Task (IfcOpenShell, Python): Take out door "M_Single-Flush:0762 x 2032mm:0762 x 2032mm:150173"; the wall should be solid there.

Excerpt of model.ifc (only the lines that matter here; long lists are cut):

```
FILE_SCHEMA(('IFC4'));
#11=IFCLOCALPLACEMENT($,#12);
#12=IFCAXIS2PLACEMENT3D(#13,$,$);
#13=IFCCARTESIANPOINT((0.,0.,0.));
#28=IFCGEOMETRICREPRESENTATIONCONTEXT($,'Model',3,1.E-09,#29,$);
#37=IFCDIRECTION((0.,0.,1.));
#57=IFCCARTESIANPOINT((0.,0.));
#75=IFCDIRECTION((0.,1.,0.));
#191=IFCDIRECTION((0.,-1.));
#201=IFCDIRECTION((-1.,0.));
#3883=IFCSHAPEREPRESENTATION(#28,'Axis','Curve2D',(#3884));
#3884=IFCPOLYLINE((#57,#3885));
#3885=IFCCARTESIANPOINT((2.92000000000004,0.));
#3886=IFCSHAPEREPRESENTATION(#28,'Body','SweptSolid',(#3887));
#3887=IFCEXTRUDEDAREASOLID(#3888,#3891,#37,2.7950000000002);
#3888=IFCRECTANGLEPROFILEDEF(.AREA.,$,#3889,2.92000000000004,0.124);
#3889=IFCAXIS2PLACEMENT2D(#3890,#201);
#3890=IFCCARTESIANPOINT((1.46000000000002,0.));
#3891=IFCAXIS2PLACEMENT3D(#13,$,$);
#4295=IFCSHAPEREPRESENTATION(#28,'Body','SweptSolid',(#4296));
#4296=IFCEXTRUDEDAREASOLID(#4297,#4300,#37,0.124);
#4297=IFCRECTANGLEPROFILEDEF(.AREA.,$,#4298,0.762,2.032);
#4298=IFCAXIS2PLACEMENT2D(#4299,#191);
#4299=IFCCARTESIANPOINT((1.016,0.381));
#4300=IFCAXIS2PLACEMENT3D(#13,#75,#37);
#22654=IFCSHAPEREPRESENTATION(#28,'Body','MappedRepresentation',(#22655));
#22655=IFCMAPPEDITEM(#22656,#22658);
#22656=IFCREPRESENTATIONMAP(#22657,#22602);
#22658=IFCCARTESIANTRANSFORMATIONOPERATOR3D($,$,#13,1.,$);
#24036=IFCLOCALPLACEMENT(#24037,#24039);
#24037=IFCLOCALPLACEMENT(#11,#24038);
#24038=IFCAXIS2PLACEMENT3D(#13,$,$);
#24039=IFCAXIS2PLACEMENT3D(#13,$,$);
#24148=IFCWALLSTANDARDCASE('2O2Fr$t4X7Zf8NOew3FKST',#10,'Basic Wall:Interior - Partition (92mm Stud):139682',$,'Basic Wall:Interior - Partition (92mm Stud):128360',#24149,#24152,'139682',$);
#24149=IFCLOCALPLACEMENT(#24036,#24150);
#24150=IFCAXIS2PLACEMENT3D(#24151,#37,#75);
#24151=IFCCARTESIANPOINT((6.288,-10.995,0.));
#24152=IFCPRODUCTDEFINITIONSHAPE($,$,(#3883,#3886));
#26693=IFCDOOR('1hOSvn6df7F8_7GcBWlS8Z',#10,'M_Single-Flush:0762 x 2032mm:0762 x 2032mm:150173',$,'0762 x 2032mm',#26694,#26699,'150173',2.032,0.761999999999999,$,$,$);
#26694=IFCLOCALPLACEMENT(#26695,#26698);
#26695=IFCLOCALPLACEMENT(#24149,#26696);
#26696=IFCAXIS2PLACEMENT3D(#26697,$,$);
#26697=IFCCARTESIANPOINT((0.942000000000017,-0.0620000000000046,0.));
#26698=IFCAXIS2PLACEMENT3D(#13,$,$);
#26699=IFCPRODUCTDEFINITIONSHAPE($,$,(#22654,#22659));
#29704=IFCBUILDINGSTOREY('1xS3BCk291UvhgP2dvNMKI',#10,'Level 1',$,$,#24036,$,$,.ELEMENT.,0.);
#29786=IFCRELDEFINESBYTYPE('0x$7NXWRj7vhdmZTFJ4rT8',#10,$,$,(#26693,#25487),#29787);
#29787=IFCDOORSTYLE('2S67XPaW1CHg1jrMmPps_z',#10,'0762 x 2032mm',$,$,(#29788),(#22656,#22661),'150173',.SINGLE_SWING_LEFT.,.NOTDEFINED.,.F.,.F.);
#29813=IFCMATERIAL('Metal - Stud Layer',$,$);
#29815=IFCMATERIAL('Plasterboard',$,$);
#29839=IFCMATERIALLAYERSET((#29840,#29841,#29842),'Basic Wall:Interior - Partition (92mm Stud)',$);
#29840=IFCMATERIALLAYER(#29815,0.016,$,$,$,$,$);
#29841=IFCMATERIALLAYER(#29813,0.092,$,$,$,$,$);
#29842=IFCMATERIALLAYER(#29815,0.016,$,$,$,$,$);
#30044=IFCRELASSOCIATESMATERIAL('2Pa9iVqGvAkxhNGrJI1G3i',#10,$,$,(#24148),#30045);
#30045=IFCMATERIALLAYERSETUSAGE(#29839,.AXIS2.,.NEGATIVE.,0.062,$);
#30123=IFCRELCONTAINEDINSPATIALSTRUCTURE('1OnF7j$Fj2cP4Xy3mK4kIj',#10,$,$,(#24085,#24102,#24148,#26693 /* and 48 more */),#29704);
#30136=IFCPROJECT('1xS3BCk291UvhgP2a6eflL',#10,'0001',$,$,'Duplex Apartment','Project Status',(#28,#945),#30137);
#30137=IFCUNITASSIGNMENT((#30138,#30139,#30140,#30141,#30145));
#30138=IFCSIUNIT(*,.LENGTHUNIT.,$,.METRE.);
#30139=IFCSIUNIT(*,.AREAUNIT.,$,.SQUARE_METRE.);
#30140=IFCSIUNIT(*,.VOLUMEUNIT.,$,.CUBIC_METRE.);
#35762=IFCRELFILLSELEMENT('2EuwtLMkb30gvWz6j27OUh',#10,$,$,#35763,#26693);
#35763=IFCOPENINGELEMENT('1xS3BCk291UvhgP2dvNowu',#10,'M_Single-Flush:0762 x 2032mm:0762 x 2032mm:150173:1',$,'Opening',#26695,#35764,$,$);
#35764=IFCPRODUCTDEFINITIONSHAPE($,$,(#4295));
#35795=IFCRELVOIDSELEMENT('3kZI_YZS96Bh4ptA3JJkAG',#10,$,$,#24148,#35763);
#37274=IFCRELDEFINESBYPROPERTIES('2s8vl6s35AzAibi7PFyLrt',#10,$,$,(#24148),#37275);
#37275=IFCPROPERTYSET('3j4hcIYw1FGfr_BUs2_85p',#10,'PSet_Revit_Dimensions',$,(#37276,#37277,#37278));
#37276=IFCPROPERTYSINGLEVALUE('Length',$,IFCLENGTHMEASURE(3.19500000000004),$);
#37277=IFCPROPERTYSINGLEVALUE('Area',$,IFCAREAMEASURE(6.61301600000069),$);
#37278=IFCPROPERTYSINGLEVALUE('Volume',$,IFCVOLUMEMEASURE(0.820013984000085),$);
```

```python
import ifcopenshell
import ifcopenshell.api.feature
import ifcopenshell.api.pset
import ifcopenshell.api.root
import ifcopenshell.geom
import ifcopenshell.util.element
import ifcopenshell.util.shape
import ifcopenshell.util.unit

model = ifcopenshell.open("model.ifc")
area_scale = ifcopenshell.util.unit.calculate_unit_scale(model, "AREAUNIT")
volume_scale = ifcopenshell.util.unit.calculate_unit_scale(model, "VOLUMEUNIT")
settings = ifcopenshell.geom.settings()


def volume(element):
    """Net volume in cubic metres, openings subtracted."""
    shape = ifcopenshell.geom.create_shape(settings, element)
    return ifcopenshell.util.shape.get_volume(shape.geometry)


door = model.by_guid("1hOSvn6df7F8_7GcBWlS8Z")
opening = door.FillsVoids[0].RelatingOpeningElement
wall = opening.VoidsElements[0].RelatingBuildingElement
before = volume(wall)

ifcopenshell.api.root.remove_product(model, product=door)
ifcopenshell.api.feature.remove_feature(model, feature=opening)

after = volume(wall)
thickness = 0.124  # wall thickness in metres

# Update the wall's stored quantities.
pset = model.by_id(ifcopenshell.util.element.get_pset(wall, "PSet_Revit_Dimensions", should_inherit=False)["id"])
ifcopenshell.api.pset.edit_pset(model, pset=pset, properties={
    "Area": model.create_entity("IfcAreaMeasure", after / thickness / area_scale),
    "Volume": model.create_entity("IfcVolumeMeasure", after / volume_scale),
})

print(f"wall volume {before:.3f} -> {after:.3f} m3")

model.write("model_updated.ifc")
```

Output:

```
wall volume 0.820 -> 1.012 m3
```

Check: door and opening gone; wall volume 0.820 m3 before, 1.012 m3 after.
